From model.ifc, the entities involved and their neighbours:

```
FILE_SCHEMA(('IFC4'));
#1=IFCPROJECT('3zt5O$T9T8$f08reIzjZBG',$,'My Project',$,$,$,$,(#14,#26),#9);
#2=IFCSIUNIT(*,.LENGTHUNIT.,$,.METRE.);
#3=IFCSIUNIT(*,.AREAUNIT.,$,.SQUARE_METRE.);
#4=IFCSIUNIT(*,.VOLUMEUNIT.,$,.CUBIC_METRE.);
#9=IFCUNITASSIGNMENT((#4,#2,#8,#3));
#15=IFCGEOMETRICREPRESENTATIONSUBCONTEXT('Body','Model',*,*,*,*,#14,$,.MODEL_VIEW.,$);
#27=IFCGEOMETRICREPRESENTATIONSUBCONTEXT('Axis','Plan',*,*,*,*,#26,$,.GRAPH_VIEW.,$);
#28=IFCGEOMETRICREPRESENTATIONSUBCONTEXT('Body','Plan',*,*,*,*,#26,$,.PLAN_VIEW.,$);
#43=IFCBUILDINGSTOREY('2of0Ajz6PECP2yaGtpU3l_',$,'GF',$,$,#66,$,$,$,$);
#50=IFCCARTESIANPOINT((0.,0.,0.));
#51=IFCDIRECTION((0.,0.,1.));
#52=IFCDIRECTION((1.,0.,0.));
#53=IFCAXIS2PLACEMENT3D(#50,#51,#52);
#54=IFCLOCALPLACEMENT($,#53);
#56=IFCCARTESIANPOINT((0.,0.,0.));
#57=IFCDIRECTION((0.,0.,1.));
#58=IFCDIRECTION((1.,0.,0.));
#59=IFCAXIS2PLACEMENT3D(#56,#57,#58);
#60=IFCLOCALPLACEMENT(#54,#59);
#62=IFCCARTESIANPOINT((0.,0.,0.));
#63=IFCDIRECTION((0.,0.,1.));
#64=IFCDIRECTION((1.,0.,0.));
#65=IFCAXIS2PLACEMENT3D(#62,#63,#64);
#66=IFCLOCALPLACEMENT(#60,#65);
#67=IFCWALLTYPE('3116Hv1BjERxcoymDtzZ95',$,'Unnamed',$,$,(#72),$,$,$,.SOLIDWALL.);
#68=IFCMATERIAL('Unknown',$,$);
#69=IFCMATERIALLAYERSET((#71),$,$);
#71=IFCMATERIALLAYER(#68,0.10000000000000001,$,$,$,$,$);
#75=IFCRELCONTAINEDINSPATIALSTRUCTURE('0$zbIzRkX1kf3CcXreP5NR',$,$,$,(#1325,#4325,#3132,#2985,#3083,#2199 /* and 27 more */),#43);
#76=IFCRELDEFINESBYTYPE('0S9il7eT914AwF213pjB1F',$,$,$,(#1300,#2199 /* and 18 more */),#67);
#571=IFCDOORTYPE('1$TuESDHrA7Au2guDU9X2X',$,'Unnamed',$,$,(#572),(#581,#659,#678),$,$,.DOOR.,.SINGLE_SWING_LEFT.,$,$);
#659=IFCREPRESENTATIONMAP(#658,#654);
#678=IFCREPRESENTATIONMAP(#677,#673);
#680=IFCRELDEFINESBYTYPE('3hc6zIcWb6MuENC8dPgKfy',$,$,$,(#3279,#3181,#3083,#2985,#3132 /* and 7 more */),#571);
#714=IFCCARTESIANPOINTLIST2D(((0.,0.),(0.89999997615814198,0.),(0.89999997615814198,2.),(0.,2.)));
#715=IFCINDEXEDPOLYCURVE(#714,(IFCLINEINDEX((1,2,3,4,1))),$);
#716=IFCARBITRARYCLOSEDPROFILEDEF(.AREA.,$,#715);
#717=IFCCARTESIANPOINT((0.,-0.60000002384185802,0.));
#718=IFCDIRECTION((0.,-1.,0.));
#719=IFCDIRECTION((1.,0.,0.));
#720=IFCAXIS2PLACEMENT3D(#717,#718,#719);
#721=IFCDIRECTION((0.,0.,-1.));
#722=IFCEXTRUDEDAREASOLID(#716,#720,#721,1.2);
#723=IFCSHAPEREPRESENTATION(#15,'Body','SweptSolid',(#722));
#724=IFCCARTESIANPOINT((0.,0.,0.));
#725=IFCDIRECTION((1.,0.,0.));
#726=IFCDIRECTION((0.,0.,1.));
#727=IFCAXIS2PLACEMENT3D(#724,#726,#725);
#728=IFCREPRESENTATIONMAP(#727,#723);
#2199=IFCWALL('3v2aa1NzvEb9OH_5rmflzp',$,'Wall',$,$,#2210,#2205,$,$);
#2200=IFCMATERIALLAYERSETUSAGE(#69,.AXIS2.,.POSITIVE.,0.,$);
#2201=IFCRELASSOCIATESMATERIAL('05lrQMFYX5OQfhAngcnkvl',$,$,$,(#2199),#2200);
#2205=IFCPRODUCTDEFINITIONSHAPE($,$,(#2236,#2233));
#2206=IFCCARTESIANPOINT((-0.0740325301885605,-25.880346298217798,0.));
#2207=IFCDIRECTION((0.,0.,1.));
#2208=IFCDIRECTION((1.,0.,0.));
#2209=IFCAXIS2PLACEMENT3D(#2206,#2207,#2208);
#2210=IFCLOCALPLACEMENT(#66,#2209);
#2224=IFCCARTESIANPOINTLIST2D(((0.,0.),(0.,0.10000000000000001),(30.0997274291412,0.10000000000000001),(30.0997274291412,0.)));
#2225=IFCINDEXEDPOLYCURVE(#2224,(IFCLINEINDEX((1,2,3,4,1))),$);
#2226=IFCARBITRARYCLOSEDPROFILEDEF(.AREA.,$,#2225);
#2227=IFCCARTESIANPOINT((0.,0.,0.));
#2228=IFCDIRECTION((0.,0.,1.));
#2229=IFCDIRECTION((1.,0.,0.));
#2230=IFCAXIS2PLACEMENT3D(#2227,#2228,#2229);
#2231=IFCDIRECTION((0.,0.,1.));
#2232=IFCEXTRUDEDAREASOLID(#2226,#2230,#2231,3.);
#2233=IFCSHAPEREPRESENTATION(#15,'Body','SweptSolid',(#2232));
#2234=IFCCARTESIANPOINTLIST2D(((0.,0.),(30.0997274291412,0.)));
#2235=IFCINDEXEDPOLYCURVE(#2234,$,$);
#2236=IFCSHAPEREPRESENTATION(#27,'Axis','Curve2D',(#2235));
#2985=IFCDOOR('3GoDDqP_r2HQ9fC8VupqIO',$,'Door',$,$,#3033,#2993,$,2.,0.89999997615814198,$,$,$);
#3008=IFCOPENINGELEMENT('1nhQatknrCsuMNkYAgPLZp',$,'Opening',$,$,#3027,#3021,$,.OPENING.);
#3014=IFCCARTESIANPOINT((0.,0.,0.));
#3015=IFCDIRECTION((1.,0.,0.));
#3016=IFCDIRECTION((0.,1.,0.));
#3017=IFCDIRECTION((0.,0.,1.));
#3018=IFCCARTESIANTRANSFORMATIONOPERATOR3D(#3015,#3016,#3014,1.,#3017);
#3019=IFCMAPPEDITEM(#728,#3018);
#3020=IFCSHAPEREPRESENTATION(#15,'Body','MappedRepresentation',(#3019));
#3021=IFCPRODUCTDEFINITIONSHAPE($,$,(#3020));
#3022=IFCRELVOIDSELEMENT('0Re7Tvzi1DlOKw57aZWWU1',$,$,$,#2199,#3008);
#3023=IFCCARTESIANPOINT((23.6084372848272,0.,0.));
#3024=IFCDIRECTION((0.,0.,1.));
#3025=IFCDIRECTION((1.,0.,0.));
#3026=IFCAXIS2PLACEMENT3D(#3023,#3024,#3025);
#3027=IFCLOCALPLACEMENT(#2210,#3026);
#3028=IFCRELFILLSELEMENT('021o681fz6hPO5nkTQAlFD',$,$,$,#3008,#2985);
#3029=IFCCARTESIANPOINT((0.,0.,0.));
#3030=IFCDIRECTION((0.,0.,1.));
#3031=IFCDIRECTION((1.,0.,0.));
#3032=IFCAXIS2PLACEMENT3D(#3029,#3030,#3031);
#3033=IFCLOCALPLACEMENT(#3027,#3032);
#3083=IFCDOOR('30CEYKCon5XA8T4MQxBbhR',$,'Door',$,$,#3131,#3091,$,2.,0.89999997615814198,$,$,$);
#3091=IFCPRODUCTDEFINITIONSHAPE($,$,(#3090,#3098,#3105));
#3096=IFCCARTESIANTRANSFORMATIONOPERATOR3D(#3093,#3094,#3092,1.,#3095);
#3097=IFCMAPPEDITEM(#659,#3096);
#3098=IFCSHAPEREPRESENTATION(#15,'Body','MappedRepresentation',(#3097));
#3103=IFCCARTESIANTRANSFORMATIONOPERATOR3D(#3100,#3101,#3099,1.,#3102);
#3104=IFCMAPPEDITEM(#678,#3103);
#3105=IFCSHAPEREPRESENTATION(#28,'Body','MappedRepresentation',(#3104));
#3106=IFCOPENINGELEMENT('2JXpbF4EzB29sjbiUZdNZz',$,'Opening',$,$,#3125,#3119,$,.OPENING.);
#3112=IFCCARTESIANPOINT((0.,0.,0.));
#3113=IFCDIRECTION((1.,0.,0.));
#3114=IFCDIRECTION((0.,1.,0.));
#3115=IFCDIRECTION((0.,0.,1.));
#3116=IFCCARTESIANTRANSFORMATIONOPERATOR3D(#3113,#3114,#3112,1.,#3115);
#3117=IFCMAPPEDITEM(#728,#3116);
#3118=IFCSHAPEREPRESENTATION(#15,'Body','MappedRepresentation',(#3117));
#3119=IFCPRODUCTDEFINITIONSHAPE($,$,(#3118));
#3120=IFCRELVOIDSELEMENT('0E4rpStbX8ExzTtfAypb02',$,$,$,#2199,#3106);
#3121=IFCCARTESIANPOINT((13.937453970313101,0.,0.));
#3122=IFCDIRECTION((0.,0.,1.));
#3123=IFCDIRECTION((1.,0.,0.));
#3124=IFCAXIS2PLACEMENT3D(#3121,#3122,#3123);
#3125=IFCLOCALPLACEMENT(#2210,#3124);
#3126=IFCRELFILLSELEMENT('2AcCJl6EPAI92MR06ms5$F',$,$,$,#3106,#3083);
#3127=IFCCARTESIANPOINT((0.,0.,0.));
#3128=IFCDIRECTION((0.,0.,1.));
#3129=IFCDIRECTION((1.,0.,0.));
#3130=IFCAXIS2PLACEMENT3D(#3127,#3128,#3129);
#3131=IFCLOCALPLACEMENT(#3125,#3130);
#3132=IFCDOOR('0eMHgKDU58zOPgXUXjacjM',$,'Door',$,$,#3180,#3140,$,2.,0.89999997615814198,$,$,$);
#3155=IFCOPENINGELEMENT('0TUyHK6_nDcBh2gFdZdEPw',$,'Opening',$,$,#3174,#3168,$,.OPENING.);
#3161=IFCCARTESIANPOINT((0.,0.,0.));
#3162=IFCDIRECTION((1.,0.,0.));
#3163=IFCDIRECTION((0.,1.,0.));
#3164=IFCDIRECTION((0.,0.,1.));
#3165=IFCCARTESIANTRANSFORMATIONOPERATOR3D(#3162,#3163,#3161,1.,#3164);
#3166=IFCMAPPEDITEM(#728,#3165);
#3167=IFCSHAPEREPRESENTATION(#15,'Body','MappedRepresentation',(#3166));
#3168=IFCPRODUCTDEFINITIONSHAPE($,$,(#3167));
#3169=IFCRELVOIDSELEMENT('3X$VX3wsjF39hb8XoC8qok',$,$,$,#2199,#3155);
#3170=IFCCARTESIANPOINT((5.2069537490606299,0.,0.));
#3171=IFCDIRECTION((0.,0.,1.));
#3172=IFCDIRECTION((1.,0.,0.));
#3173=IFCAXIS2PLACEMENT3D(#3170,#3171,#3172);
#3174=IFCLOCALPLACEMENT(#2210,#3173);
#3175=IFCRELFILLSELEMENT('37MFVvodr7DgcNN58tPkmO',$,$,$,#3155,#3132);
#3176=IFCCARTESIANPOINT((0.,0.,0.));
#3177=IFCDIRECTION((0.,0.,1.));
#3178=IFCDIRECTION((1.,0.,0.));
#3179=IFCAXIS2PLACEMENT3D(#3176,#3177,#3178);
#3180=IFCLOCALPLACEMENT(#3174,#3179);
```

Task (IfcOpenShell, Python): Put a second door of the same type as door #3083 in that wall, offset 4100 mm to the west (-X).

```python
import ifcopenshell
import ifcopenshell.api.feature
import ifcopenshell.api.geometry
import ifcopenshell.api.root
import ifcopenshell.geom
import ifcopenshell.util.element
import ifcopenshell.util.placement
import ifcopenshell.util.shape
import ifcopenshell.util.unit

model = ifcopenshell.open("model.ifc")
unit_scale = ifcopenshell.util.unit.calculate_unit_scale(model)
settings = ifcopenshell.geom.settings()


def volume(element):
    """Net volume in cubic metres, openings subtracted."""
    shape = ifcopenshell.geom.create_shape(settings, element)
    return ifcopenshell.util.shape.get_volume(shape.geometry)


door = model.by_guid("30CEYKCon5XA8T4MQxBbhR")
opening = door.FillsVoids[0].RelatingOpeningElement
wall = opening.VoidsElements[0].RelatingBuildingElement
before = volume(wall)
shift = ifcopenshell.util.placement.get_local_placement(wall.ObjectPlacement)[:3, 0] * -4.1 / unit_scale

# copy_class copies the void relationship, type, container and properties, but no geometry.
new_opening = ifcopenshell.api.root.copy_class(model, product=opening)
new_opening.Representation = ifcopenshell.util.element.copy_deep(
    model, opening.Representation, exclude=["IfcGeometricRepresentationContext", "IfcRepresentationMap"]
)
new_door = ifcopenshell.api.root.copy_class(model, product=door)
new_door.Representation = ifcopenshell.util.element.copy_deep(
    model, door.Representation, exclude=["IfcGeometricRepresentationContext", "IfcRepresentationMap"]
)
ifcopenshell.api.feature.add_filling(model, opening=new_opening, element=new_door)

for old, new in ((opening, new_opening), (door, new_door)):
    matrix = ifcopenshell.util.placement.get_local_placement(old.ObjectPlacement)
    matrix[:3, 3] += shift
    ifcopenshell.api.geometry.edit_object_placement(model, product=new, matrix=matrix, is_si=False)

after = volume(wall)

print(f"wall volume {before:.3f} -> {after:.3f} m3")

model.write("model-out.ifc")
```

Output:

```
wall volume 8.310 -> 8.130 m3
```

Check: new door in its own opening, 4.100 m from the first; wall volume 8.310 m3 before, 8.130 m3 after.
